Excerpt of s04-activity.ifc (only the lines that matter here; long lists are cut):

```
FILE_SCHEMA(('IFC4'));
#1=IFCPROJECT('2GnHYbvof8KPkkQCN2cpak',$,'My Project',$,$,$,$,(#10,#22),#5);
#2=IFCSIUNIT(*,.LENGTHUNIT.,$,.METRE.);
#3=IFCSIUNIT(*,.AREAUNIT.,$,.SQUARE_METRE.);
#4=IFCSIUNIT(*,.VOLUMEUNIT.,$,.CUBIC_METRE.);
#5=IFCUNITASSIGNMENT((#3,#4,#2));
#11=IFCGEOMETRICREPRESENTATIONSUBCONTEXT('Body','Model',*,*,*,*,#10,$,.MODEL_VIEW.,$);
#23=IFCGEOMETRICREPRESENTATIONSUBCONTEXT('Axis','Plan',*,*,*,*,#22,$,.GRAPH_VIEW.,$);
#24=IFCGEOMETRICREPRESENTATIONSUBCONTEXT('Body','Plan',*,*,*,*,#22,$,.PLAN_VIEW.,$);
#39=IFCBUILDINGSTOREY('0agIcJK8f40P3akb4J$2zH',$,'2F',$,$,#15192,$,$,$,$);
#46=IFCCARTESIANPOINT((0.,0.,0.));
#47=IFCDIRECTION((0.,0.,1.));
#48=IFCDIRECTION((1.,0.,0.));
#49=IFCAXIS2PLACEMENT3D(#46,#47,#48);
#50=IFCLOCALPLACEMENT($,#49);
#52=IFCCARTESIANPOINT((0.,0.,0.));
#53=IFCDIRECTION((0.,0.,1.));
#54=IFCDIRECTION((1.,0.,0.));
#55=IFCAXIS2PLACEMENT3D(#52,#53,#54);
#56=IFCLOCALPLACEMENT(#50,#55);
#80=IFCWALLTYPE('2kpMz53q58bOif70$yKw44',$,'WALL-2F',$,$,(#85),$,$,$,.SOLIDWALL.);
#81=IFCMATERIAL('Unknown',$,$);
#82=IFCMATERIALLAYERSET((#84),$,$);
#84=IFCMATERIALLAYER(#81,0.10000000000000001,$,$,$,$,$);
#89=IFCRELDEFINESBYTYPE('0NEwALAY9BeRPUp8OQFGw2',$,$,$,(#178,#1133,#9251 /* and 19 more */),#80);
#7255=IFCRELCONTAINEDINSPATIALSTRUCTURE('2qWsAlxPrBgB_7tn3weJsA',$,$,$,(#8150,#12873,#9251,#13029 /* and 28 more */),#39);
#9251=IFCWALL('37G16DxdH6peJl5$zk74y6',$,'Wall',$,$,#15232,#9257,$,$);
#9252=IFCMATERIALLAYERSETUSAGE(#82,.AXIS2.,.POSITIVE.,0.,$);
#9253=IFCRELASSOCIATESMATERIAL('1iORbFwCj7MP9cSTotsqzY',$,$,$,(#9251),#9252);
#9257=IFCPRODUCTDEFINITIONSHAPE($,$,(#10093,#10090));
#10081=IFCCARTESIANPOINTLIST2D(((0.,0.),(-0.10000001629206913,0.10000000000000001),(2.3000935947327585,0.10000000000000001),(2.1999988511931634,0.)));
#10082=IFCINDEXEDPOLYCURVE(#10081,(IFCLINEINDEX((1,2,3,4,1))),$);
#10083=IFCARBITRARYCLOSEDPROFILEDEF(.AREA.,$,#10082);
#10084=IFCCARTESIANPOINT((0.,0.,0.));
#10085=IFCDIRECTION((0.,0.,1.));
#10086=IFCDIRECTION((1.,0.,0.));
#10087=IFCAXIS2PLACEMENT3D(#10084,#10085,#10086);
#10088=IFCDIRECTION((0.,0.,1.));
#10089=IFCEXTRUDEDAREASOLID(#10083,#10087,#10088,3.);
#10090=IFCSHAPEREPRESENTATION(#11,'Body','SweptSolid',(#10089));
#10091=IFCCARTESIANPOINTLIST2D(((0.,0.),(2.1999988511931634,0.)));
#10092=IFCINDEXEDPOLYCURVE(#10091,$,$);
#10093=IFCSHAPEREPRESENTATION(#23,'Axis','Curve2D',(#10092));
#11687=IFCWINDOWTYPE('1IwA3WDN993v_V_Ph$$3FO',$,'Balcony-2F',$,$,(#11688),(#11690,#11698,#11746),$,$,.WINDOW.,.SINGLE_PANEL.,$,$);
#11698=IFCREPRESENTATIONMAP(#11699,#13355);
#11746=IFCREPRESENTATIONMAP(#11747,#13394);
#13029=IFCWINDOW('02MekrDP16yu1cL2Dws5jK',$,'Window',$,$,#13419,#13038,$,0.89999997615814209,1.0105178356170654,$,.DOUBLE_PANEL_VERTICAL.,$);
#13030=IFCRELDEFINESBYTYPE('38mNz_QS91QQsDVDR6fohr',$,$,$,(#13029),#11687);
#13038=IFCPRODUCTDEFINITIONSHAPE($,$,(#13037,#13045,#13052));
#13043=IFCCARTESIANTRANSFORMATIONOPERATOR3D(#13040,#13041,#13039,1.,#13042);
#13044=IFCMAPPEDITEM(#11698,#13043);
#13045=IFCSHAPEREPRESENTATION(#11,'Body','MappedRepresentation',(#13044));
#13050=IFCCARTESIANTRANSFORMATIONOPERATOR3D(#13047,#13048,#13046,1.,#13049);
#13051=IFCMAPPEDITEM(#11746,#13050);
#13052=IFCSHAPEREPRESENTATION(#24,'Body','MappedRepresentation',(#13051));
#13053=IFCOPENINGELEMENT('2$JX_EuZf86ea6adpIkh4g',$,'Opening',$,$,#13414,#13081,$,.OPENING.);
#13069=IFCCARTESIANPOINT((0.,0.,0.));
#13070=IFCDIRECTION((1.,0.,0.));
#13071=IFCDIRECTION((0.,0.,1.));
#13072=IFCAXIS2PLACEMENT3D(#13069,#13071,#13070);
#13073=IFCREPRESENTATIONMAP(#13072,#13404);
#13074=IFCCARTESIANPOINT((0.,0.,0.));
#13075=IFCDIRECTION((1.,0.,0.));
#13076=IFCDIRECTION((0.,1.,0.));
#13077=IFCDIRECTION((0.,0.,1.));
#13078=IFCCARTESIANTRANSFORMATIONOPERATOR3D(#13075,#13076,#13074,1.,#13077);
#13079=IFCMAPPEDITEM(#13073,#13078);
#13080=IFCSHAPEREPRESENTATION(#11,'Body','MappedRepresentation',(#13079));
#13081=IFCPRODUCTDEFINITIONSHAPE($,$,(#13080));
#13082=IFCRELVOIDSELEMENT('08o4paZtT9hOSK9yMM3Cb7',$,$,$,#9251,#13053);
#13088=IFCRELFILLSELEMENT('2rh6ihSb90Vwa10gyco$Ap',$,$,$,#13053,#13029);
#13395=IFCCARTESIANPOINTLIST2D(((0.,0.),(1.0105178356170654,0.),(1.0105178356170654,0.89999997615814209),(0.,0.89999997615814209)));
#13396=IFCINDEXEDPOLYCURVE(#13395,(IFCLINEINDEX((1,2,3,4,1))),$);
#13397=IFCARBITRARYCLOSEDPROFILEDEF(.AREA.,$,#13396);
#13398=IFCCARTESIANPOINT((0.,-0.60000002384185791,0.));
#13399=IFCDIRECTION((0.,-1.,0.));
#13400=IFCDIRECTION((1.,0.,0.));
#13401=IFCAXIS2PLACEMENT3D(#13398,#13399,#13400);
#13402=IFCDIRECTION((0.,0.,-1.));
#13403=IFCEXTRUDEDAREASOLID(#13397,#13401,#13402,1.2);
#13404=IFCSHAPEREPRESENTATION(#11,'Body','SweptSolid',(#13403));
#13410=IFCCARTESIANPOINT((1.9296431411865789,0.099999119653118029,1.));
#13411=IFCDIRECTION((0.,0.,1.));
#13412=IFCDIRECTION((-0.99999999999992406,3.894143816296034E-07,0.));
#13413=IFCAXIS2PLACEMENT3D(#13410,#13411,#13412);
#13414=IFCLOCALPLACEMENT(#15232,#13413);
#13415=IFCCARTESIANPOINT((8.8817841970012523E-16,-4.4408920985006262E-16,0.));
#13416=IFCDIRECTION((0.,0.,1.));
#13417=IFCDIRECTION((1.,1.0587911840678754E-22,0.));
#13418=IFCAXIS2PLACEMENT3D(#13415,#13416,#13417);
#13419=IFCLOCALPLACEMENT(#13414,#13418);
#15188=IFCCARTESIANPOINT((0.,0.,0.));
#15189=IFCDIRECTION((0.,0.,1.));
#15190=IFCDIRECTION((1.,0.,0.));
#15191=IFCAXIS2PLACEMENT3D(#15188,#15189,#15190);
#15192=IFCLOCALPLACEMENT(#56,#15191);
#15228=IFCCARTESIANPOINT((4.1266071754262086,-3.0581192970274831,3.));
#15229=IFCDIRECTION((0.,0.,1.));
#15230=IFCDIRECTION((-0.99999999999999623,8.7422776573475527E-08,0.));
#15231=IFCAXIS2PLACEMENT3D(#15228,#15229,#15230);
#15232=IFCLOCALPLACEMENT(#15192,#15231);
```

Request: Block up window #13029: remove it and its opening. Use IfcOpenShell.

```python
import ifcopenshell
import ifcopenshell.api.feature
import ifcopenshell.api.root
import ifcopenshell.geom
import ifcopenshell.util.shape

model = ifcopenshell.open("s04-activity.ifc")
settings = ifcopenshell.geom.settings()


def volume(element):
    """Net volume in cubic metres, openings subtracted."""
    shape = ifcopenshell.geom.create_shape(settings, element)
    return ifcopenshell.util.shape.get_volume(shape.geometry)


window = model.by_guid("02MekrDP16yu1cL2Dws5jK")
opening = window.FillsVoids[0].RelatingOpeningElement
wall = opening.VoidsElements[0].RelatingBuildingElement
before = volume(wall)

ifcopenshell.api.root.remove_product(model, product=window)
ifcopenshell.api.feature.remove_feature(model, feature=opening)

after = volume(wall)

print(f"wall volume {before:.3f} -> {after:.3f} m3")

model.write("s04-activity_rev.ifc")
```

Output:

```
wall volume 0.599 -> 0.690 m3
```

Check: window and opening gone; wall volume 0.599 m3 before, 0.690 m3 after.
